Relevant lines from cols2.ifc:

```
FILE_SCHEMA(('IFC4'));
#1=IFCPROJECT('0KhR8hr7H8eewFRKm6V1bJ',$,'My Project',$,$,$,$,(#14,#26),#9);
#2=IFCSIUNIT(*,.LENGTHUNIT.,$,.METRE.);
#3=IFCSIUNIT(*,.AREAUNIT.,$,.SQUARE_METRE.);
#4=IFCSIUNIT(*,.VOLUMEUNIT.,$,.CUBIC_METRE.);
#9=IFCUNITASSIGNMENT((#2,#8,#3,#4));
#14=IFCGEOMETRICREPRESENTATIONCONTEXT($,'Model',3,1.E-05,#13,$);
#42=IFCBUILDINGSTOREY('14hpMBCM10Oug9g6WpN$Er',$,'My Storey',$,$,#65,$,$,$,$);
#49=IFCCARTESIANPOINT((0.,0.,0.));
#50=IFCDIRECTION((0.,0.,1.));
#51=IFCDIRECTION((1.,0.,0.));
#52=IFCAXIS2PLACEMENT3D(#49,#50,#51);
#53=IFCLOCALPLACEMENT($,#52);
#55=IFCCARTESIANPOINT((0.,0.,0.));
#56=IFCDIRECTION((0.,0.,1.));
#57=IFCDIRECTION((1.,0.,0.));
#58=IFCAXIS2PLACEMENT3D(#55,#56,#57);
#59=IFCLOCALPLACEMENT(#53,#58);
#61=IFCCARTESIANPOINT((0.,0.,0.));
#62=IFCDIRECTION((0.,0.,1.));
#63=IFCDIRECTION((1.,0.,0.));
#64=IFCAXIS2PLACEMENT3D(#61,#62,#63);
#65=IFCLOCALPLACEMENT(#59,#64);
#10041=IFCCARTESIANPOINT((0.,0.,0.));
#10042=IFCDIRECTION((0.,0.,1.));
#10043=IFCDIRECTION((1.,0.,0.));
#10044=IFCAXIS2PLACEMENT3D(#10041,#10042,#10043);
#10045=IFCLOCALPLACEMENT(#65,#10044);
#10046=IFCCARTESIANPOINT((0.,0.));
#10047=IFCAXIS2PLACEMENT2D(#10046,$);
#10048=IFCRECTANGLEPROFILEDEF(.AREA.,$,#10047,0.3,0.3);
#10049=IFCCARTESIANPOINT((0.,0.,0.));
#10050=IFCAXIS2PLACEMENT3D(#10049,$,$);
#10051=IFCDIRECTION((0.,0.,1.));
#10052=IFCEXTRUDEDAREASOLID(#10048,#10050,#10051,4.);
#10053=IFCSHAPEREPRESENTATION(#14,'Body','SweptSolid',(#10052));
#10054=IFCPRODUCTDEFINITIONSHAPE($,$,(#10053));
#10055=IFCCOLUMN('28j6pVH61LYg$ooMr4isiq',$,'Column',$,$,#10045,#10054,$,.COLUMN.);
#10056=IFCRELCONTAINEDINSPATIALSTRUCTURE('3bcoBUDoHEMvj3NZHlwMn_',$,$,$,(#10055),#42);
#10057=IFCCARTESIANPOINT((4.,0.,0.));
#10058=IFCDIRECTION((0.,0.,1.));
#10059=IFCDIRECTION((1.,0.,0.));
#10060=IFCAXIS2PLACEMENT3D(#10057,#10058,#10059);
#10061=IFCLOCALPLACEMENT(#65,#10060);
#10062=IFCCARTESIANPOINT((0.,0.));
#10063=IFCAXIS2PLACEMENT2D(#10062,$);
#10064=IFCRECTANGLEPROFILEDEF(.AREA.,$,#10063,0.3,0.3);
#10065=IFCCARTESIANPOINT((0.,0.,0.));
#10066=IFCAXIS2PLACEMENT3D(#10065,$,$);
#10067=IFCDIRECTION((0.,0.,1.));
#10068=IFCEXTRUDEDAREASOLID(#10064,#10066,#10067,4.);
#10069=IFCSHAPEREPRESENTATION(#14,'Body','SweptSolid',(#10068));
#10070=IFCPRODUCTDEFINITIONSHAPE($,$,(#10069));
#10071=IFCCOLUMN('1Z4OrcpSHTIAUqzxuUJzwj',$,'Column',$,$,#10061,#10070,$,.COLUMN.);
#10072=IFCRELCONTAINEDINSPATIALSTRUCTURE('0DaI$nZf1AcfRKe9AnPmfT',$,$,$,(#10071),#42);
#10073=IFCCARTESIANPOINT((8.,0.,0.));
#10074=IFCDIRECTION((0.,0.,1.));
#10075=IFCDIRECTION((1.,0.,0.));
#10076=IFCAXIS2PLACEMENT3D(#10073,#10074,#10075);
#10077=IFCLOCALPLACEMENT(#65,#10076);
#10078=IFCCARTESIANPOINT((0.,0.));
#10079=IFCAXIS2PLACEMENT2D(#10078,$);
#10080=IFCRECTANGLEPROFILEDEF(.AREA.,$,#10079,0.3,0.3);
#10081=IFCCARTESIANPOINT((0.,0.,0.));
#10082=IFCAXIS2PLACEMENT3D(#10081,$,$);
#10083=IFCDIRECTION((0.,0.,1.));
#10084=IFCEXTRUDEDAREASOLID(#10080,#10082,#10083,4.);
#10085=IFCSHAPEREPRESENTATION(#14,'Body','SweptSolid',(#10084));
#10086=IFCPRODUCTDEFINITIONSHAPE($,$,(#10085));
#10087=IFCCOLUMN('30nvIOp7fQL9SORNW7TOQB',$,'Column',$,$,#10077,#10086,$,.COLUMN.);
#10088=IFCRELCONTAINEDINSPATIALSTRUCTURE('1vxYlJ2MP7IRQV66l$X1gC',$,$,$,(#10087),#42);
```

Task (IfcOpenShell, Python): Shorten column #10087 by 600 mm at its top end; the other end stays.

```python
import ifcopenshell
import ifcopenshell.util.unit

model = ifcopenshell.open("cols2.ifc")
unit_scale = ifcopenshell.util.unit.calculate_unit_scale(model)

member = model.by_id(10087)
change = -0.6 / unit_scale

# The extrusion runs towards the end named, so only its depth changes.
body = next(r for r in member.Representation.Representations if r.RepresentationIdentifier == "Body")
solid = body.Items[0]
old_length = solid.Depth
solid.Depth += change

print(f"length {old_length:g} -> {solid.Depth:g}")

model.write("cols2-out.ifc")
```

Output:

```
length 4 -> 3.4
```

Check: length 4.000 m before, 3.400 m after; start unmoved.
